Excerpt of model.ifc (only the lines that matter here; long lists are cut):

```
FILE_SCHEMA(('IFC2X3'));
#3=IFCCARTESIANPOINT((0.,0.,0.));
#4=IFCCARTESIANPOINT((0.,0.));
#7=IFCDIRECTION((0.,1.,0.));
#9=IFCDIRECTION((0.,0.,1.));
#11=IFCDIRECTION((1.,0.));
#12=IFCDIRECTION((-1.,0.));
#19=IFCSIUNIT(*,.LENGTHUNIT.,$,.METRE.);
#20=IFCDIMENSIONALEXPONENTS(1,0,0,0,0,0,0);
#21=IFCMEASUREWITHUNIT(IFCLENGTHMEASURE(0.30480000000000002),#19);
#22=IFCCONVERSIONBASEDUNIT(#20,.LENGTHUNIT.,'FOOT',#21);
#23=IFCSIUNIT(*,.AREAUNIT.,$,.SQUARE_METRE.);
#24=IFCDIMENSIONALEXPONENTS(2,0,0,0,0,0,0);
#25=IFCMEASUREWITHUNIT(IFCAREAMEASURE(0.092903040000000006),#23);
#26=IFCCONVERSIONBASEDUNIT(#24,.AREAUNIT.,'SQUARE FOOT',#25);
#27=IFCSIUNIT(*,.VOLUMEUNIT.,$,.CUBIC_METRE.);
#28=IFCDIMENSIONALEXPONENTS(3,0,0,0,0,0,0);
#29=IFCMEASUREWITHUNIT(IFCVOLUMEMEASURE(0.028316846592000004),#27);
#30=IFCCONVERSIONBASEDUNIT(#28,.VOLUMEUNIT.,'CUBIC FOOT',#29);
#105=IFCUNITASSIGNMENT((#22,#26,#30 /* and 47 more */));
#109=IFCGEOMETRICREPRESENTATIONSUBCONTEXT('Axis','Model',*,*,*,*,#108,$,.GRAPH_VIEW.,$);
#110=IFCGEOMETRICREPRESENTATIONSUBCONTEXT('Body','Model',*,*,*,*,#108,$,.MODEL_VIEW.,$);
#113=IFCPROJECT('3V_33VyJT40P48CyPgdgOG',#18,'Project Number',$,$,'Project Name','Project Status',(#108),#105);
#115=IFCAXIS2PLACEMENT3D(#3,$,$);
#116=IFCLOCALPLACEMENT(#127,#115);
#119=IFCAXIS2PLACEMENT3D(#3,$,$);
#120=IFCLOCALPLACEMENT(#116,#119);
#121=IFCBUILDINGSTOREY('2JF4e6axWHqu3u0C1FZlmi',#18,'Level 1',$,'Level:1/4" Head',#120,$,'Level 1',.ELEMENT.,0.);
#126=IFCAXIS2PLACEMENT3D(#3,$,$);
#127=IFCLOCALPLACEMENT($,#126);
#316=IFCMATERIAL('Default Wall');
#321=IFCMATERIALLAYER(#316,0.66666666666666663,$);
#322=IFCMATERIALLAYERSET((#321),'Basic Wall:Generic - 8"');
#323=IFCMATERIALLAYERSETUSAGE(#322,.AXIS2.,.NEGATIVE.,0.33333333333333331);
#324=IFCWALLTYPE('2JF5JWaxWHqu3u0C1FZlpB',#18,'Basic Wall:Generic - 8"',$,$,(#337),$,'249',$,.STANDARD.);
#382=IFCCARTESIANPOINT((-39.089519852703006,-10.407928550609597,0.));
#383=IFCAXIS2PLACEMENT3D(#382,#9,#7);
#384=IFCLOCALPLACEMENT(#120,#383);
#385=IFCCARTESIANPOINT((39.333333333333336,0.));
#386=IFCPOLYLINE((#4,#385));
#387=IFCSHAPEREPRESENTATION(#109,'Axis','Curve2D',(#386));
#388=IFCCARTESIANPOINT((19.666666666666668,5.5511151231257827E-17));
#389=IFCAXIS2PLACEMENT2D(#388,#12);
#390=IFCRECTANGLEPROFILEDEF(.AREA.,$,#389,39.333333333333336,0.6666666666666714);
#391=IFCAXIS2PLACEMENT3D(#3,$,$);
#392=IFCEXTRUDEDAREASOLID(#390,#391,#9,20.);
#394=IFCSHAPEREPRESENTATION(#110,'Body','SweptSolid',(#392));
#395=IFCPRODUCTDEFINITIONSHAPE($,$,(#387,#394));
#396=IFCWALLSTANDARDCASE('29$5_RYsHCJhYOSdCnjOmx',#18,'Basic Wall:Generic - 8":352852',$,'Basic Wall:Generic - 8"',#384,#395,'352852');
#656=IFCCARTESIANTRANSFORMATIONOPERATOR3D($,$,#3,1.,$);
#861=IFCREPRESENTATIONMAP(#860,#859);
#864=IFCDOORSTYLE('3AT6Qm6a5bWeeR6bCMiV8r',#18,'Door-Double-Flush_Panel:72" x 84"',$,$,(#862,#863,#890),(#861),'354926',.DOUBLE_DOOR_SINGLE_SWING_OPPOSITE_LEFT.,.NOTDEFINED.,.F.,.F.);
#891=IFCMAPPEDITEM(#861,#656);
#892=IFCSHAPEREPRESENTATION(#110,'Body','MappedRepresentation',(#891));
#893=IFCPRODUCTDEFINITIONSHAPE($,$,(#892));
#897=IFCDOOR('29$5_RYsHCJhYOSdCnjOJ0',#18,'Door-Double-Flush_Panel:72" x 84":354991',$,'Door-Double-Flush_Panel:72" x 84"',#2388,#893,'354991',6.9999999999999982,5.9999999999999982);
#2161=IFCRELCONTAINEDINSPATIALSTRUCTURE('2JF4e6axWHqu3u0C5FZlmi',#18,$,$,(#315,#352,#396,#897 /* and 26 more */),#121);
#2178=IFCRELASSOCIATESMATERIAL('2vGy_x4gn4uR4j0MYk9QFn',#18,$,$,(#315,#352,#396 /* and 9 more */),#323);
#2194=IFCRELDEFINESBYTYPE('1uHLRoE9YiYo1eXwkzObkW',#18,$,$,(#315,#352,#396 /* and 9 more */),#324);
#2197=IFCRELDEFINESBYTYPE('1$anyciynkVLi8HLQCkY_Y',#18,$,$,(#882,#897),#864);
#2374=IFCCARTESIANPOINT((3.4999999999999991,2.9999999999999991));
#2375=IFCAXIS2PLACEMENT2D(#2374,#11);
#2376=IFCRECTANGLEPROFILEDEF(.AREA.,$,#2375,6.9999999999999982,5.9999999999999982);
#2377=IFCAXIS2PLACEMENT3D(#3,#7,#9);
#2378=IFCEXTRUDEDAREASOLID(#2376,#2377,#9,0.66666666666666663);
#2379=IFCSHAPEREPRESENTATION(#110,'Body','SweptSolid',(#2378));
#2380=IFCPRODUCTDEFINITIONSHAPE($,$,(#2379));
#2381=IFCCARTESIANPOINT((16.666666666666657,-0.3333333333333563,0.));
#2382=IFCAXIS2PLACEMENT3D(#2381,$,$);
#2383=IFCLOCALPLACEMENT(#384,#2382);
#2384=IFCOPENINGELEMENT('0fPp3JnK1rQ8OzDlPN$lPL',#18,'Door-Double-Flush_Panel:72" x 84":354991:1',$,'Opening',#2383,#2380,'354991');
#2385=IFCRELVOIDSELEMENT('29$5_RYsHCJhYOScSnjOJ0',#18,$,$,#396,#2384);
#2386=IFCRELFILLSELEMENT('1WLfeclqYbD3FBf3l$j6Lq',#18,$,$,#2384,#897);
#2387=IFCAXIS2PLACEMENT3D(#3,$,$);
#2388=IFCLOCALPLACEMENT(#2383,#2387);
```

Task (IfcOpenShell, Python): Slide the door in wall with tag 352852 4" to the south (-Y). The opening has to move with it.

```python
import ifcopenshell
import ifcopenshell.api.geometry
import ifcopenshell.util.placement
import ifcopenshell.util.unit

model = ifcopenshell.open("model.ifc")
unit_scale = ifcopenshell.util.unit.calculate_unit_scale(model)

door = model.by_id(897)
opening = door.FillsVoids[0].RelatingOpeningElement
wall = opening.VoidsElements[0].RelatingBuildingElement

wall_matrix = ifcopenshell.util.placement.get_local_placement(wall.ObjectPlacement)
shift = wall_matrix[:3, 0] * -4 * 0.0254 / unit_scale
before = ifcopenshell.util.placement.get_local_placement(door.ObjectPlacement)[:3, 3].copy()

# The door is placed relative to its opening, so it follows when the opening moves.
matrix = ifcopenshell.util.placement.get_local_placement(opening.ObjectPlacement)
matrix[:3, 3] += shift
ifcopenshell.api.geometry.edit_object_placement(
    model, product=opening, matrix=matrix, is_si=False, should_transform_children=True
)

after = ifcopenshell.util.placement.get_local_placement(door.ObjectPlacement)[:3, 3]
print("door moved by", (after - before).round(3) + 0.0)

model.write("model_updated.ifc")
```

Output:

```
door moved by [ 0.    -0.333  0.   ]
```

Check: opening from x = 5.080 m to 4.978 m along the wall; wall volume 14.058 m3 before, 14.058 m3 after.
